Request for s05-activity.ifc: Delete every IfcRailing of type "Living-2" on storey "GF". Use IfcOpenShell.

First a look at what the model holds.

```python
import ifcopenshell
import ifcopenshell.util.element

model = ifcopenshell.open("s05-activity.ifc")
print(model.schema)
storey = next(s for s in model.by_type("IfcBuildingStorey") if s.Name == "GF")
railings = [e for e in ifcopenshell.util.element.get_decomposition(storey) if e.is_a("IfcRailing")]
seen = {}
for e in railings:
    element_type = ifcopenshell.util.element.get_type(e)
    name = element_type.Name if element_type not in (None, e) else None
    seen[name] = seen.get(name, 0) + 1
for name, count in sorted(seen.items(), key=str):
    print(count, "x", name)
```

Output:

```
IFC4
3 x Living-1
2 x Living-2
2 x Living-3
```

```python
import ifcopenshell
import ifcopenshell.api.root
import ifcopenshell.util.element

model = ifcopenshell.open("s05-activity.ifc")

storey = next(s for s in model.by_type("IfcBuildingStorey") if s.Name == "GF")
railings = [e for e in ifcopenshell.util.element.get_decomposition(storey) if e.is_a("IfcRailing")]
targets = [e for e in railings if (t := ifcopenshell.util.element.get_type(e)) not in (None, e) and t.Name == "Living-2"]

for e in targets:
    ifcopenshell.api.root.remove_product(model, product=e)
print(len(targets), "removed")

model.write("s05-activity_updated.ifc")
```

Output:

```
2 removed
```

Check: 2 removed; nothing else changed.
